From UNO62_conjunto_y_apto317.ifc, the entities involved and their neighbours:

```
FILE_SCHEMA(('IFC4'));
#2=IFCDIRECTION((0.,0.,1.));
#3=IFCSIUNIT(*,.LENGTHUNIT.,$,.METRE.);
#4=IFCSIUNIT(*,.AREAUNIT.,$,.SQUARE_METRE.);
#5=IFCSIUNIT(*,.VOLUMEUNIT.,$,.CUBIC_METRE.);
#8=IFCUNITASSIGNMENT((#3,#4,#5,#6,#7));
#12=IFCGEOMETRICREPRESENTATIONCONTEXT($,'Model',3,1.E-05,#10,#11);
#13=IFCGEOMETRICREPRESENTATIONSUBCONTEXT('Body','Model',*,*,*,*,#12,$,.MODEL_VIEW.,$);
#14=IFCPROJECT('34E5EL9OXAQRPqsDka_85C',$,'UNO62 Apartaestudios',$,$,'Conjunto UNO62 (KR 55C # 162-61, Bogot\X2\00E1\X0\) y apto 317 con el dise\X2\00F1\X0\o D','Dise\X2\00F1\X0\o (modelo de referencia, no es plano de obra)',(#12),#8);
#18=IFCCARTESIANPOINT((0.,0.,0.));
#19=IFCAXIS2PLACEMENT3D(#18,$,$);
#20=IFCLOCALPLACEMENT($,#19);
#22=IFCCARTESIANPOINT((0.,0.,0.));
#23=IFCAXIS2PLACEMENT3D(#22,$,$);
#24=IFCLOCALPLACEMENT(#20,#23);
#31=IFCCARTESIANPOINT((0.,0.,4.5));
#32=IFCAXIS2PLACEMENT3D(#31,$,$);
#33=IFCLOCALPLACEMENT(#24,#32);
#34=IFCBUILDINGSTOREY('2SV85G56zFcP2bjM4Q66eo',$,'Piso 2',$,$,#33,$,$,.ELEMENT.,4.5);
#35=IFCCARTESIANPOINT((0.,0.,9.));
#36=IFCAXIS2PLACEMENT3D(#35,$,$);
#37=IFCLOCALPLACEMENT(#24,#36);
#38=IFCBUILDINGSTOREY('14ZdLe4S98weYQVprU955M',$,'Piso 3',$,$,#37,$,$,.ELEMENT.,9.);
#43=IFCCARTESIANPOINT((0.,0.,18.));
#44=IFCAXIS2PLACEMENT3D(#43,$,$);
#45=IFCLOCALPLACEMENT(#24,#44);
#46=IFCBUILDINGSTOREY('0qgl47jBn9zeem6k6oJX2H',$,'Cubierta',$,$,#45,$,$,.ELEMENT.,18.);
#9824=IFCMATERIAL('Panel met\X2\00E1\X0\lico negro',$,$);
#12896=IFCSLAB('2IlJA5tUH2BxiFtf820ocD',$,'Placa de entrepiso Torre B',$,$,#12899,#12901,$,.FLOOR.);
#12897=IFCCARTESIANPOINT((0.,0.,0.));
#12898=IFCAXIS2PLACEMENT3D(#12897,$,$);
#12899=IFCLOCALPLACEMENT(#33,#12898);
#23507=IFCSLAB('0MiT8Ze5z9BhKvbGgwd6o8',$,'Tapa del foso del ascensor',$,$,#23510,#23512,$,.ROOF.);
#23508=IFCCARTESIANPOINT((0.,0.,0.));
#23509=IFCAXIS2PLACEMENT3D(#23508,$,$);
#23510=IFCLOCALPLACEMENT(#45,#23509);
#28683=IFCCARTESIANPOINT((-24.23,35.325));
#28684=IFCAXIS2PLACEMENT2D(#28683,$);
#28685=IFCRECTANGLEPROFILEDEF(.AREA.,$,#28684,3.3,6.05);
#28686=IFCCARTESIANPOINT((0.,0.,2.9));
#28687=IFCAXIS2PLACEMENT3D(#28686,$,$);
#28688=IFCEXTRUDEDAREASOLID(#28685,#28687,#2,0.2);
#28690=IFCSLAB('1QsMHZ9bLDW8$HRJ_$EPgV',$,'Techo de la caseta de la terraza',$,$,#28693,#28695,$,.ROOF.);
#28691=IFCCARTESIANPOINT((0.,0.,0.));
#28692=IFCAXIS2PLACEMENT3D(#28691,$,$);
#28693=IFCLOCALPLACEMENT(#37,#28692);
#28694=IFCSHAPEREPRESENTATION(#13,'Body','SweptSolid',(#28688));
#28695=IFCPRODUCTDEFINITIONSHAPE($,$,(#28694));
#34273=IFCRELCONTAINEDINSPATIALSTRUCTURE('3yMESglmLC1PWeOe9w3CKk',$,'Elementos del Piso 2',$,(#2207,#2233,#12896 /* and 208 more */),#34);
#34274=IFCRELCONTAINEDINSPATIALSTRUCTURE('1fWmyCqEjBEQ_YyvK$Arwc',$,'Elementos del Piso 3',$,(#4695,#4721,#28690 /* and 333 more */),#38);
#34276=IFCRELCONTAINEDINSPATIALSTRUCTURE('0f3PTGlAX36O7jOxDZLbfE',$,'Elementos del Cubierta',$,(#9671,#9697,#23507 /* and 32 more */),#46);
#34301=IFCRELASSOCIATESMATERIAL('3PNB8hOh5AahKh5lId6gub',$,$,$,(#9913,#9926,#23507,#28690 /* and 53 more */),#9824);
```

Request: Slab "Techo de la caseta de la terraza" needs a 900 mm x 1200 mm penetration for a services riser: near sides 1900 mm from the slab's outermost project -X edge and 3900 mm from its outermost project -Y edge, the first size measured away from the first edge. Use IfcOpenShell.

```python
import numpy as np
import ifcopenshell
import ifcopenshell.api.feature
import ifcopenshell.api.geometry
import ifcopenshell.api.root
import ifcopenshell.geom
import ifcopenshell.util.placement
import ifcopenshell.util.representation
import ifcopenshell.util.shape
import ifcopenshell.util.unit

model = ifcopenshell.open("UNO62_conjunto_y_apto317.ifc")
unit_scale = ifcopenshell.util.unit.calculate_unit_scale(model)
settings = ifcopenshell.geom.settings()


def volume(element):
    """Net volume in cubic metres, openings subtracted."""
    shape = ifcopenshell.geom.create_shape(settings, element)
    return ifcopenshell.util.shape.get_volume(shape.geometry)


slab = model.by_guid("1QsMHZ9bLDW8$HRJ_$EPgV")
before = volume(slab)

# Extent in the slab's own axes, in metres. The edges named are its -X and -Y sides.
slab_shape = ifcopenshell.geom.create_shape(settings, slab)
vertices = ifcopenshell.util.shape.get_vertices(slab_shape.geometry)
x_min, y_min, bottom = vertices.min(axis=0)
top = vertices[:, 2].max()

opening = ifcopenshell.api.root.create_entity(model, ifc_class="IfcOpeningElement", name="Services riser opening", predefined_type="OPENING")
context = ifcopenshell.util.representation.get_context(model, "Model", "Body", "MODEL_VIEW")
width, depth = 0.9, 1.2
outline = [(0.0, 0.0), (width, 0.0), (width, depth), (0.0, depth), (0.0, 0.0)]
# Overshoot both faces by 50 mm so the cut is clean.
shape = ifcopenshell.api.geometry.add_slab_representation(
    model, context=context, depth=top - bottom + 0.1, polyline=outline
)
ifcopenshell.api.geometry.assign_representation(model, product=opening, representation=shape)

matrix = ifcopenshell.util.placement.get_local_placement(slab.ObjectPlacement)
matrix[:, 3] = matrix @ np.append(np.array([x_min + 1.9, y_min + 3.9, bottom - 0.05]) / unit_scale, 1.0)
ifcopenshell.api.geometry.edit_object_placement(model, product=opening, matrix=matrix, is_si=False)
ifcopenshell.api.feature.add_feature(model, feature=opening, element=slab)

after = volume(slab)

print(f"slab volume {before:.3f} -> {after:.3f} m3")

model.write("UNO62_conjunto_y_apto317_updated.ifc")
```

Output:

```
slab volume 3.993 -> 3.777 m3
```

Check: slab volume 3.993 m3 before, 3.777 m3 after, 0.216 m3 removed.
